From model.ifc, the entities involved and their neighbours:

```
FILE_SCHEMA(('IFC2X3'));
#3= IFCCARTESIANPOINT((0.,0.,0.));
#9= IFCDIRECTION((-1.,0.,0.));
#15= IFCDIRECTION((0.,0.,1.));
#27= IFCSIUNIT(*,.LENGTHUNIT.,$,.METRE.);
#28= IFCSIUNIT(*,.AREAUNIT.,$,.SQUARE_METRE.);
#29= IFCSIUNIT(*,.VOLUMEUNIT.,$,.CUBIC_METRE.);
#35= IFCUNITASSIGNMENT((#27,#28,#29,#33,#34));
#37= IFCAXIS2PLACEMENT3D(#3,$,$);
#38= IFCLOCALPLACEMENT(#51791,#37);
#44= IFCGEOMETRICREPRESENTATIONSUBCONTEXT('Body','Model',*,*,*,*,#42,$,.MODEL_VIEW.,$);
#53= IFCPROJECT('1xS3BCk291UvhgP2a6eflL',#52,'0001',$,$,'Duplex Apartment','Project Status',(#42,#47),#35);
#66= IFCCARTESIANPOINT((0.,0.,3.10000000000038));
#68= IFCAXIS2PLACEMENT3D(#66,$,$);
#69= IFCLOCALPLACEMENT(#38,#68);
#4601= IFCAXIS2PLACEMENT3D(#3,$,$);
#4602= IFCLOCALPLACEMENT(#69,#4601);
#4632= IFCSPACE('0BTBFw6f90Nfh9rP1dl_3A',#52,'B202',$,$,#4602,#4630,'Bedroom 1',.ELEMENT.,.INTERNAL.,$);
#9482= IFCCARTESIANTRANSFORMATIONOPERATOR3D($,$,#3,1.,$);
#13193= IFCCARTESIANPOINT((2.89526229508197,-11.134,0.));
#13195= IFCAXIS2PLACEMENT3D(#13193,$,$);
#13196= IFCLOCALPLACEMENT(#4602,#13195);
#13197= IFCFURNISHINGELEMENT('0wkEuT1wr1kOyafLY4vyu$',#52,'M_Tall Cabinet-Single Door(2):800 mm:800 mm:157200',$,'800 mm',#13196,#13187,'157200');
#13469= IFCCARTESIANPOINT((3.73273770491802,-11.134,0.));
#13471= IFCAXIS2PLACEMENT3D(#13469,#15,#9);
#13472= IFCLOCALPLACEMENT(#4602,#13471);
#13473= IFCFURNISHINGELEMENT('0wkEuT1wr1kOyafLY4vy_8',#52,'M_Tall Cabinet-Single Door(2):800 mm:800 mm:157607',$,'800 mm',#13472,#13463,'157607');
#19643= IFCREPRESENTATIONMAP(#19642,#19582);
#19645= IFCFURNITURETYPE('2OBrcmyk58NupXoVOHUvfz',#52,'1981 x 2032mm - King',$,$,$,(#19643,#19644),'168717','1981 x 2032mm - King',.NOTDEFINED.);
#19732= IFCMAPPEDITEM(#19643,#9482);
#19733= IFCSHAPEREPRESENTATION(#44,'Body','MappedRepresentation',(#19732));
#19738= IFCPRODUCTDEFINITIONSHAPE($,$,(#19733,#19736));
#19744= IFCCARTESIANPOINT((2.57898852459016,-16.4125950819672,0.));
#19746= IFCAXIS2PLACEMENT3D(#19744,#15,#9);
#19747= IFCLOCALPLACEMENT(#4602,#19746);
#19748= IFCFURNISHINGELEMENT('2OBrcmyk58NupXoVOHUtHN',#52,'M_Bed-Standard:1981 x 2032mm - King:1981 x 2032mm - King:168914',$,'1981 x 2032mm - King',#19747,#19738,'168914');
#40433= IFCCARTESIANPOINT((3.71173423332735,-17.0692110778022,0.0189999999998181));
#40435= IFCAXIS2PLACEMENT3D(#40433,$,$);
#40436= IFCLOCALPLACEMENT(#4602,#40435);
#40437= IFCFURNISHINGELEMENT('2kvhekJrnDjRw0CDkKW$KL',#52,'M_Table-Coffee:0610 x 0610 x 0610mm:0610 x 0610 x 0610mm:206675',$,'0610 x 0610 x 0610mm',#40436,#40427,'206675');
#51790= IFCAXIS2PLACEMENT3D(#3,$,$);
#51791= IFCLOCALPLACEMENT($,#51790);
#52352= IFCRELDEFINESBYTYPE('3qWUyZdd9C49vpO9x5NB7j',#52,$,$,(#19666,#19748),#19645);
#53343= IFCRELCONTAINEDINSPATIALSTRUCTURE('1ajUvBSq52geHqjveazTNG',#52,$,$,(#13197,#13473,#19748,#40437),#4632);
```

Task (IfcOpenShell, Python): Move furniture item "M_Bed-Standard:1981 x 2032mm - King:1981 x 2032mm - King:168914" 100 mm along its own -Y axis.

```python
import ifcopenshell
import ifcopenshell.api.geometry
import ifcopenshell.util.placement

model = ifcopenshell.open("model.ifc")

item = model.by_id(19748)
matrix = ifcopenshell.util.placement.get_local_placement(item.ObjectPlacement)
matrix[:3, 3] -= matrix[:3, 1] * 0.1
ifcopenshell.api.geometry.edit_object_placement(model, product=item, matrix=matrix, is_si=False)

print(ifcopenshell.util.placement.get_local_placement(item.ObjectPlacement).round(3) + 0.0)

model.write("model-out.ifc")
```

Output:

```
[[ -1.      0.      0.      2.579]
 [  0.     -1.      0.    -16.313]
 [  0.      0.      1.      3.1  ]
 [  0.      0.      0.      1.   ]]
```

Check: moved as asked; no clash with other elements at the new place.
